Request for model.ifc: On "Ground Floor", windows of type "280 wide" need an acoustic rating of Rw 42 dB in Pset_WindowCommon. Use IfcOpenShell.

First a look at what the model holds.

```python
import ifcopenshell
import ifcopenshell.util.element

model = ifcopenshell.open("model.ifc")
print(model.schema)
storey = next(s for s in model.by_type("IfcBuildingStorey") if s.Name == "Ground Floor")
windows = [e for e in ifcopenshell.util.element.get_decomposition(storey) if e.is_a("IfcWindow")]
seen = {}
for e in windows:
    element_type = ifcopenshell.util.element.get_type(e)
    key = (element_type.Name if element_type != e and element_type else None, ifcopenshell.util.element.get_pset(e, "Pset_WindowCommon", "AcousticRating"))
    seen[key] = seen.get(key, 0) + 1
for (name, value), count in sorted(seen.items(), key=str):
    print(count, "x", name, "|", value)
```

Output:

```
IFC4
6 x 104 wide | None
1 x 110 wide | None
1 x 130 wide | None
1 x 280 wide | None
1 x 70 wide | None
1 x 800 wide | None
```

```python
import ifcopenshell
import ifcopenshell.api.pset
import ifcopenshell.util.element

model = ifcopenshell.open("model.ifc")

storey = next(s for s in model.by_type("IfcBuildingStorey") if s.Name == "Ground Floor")
windows = [e for e in ifcopenshell.util.element.get_decomposition(storey) if e.is_a("IfcWindow")]

count = 0
for e in windows:
    element_type = ifcopenshell.util.element.get_type(e)
    if element_type in (None, e) or element_type.Name != "280 wide":
        continue
    # add_pset returns the element's existing set when there is one.
    pset = ifcopenshell.api.pset.add_pset(model, product=e, name="Pset_WindowCommon")
    ifcopenshell.api.pset.edit_pset(model, pset=pset, properties={"AcousticRating": "Rw 42 dB"})
    count += 1

print(count, "windows updated")

model.write("model_edited.ifc")
```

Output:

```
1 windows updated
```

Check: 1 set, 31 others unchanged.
